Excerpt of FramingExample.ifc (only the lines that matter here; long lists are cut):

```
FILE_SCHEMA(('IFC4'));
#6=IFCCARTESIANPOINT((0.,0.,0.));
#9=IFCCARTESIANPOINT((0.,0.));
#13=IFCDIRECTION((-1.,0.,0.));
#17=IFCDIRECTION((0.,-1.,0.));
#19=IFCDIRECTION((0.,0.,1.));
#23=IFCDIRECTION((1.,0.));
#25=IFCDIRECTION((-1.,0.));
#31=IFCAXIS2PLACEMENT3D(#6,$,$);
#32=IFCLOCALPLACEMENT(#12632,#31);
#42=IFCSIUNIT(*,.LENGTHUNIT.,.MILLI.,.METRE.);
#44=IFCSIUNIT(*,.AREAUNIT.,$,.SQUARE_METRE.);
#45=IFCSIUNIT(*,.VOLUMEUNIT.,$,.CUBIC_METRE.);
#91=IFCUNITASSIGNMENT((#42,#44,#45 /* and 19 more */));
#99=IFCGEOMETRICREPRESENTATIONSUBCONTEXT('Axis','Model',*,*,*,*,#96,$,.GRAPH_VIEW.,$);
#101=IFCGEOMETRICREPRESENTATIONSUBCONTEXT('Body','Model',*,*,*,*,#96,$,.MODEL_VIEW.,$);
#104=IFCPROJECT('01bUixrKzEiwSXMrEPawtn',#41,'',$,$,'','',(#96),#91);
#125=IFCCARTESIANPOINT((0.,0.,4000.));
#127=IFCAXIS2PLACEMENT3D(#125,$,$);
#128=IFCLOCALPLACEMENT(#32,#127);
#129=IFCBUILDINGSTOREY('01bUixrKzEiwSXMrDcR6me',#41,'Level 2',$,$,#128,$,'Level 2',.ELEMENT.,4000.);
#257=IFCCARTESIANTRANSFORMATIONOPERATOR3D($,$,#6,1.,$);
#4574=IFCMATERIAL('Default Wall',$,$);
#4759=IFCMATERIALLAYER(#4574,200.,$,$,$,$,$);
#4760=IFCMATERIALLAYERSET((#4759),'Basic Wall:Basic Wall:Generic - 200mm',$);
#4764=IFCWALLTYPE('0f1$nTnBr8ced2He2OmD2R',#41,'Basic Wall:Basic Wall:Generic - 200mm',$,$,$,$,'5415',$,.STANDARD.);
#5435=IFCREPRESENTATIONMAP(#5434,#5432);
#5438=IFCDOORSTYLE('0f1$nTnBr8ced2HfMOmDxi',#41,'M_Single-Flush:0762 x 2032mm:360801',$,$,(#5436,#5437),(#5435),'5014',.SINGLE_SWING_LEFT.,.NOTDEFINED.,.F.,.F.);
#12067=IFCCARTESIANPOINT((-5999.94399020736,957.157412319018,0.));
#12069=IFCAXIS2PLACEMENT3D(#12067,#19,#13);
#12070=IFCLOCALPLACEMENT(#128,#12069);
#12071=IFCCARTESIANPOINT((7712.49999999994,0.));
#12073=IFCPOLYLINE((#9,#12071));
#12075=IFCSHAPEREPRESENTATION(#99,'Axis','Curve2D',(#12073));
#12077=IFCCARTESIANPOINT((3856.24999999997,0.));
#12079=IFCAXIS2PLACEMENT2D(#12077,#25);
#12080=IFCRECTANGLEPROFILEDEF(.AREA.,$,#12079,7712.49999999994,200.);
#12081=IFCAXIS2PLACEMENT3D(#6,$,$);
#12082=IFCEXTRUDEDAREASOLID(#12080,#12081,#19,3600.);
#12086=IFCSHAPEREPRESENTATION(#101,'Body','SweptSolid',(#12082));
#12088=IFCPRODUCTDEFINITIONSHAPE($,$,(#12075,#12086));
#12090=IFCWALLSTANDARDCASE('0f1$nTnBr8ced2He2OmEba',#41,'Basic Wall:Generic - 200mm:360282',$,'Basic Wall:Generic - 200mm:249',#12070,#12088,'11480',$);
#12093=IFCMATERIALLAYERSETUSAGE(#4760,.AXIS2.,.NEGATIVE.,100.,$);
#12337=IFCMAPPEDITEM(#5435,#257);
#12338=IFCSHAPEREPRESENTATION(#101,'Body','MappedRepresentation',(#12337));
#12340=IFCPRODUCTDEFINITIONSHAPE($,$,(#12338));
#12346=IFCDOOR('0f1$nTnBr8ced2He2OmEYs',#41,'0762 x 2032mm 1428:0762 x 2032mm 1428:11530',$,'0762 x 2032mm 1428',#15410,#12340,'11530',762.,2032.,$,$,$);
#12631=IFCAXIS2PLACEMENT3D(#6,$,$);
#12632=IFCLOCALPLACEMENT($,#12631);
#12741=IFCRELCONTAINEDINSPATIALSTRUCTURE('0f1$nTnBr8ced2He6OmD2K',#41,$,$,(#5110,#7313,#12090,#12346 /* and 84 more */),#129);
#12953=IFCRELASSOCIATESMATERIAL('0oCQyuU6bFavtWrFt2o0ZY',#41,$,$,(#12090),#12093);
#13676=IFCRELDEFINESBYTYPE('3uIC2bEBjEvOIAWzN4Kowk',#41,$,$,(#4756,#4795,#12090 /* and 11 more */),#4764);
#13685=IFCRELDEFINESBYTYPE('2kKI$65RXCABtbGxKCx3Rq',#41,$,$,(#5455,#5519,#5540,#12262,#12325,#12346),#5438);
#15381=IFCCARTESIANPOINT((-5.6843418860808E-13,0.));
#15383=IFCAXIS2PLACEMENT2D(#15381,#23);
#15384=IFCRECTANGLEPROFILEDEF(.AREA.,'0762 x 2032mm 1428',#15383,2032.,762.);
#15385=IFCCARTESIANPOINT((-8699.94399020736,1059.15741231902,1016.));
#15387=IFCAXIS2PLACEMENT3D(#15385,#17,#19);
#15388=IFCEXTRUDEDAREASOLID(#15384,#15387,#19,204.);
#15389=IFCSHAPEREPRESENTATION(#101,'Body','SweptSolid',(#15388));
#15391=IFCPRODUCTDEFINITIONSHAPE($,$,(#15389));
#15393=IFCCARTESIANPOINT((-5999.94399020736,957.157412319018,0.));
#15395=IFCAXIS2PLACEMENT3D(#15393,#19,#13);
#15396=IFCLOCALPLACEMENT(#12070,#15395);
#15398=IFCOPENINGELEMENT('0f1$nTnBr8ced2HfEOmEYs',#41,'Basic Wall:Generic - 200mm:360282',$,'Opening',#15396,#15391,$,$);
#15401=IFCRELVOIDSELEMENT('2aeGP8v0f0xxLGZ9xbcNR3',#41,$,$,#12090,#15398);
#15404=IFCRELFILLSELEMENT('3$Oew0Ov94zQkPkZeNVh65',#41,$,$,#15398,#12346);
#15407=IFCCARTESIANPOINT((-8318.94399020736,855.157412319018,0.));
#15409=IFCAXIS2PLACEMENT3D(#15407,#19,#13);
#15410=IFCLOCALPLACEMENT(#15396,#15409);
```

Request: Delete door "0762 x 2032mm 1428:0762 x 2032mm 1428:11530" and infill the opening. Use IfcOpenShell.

```python
import ifcopenshell
import ifcopenshell.api.feature
import ifcopenshell.api.root
import ifcopenshell.geom
import ifcopenshell.util.shape

model = ifcopenshell.open("FramingExample.ifc")
settings = ifcopenshell.geom.settings()


def volume(element):
    """Net volume in cubic metres, openings subtracted."""
    shape = ifcopenshell.geom.create_shape(settings, element)
    return ifcopenshell.util.shape.get_volume(shape.geometry)


door = model.by_guid("0f1$nTnBr8ced2He2OmEYs")
opening = door.FillsVoids[0].RelatingOpeningElement
wall = opening.VoidsElements[0].RelatingBuildingElement
before = volume(wall)

ifcopenshell.api.root.remove_product(model, product=door)
ifcopenshell.api.feature.remove_feature(model, feature=opening)

after = volume(wall)

print(f"wall volume {before:.3f} -> {after:.3f} m3")

model.write("FramingExample-out.ifc")
```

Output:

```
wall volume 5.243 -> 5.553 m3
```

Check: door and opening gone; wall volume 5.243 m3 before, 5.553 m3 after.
